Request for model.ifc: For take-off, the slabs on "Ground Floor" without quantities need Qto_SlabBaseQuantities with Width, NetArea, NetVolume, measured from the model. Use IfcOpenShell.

First a look at what the model holds.

```python
import ifcopenshell
import ifcopenshell.util.element
import ifcopenshell.util.unit

model = ifcopenshell.open("model.ifc")
print(model.schema)
for unit_type in ("LENGTHUNIT", "AREAUNIT", "VOLUMEUNIT"):
    print(unit_type, ifcopenshell.util.unit.calculate_unit_scale(model, unit_type))
storey = next(s for s in model.by_type("IfcBuildingStorey") if s.Name == "Ground Floor")
slabs = [e for e in ifcopenshell.util.element.get_decomposition(storey) if e.is_a("IfcSlab")]
for e in sorted(slabs, key=lambda e: e.id()):
    print(e.id(), e.is_a(), e.Name, list(ifcopenshell.util.element.get_psets(e, qtos_only=True)), sep=" | ")
```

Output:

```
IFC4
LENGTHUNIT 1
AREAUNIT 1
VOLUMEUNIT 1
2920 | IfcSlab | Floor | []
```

```python
import ifcopenshell
import ifcopenshell.api.pset
import ifcopenshell.geom
import ifcopenshell.util.element
import ifcopenshell.util.shape
import ifcopenshell.util.unit

model = ifcopenshell.open("model.ifc")
unit_scale = ifcopenshell.util.unit.calculate_unit_scale(model)
area_scale = ifcopenshell.util.unit.calculate_unit_scale(model, "AREAUNIT")
volume_scale = ifcopenshell.util.unit.calculate_unit_scale(model, "VOLUMEUNIT")
settings = ifcopenshell.geom.settings()

storey = next(s for s in model.by_type("IfcBuildingStorey") if s.Name == "Ground Floor")
slabs = [e for e in ifcopenshell.util.element.get_decomposition(storey) if e.is_a("IfcSlab")]

for e in sorted(slabs, key=lambda e: e.id()):
    if ifcopenshell.util.element.get_psets(e, qtos_only=True, should_inherit=False):
        continue
    # Geometry comes back in metres, in the element's own axes.
    shape = ifcopenshell.geom.create_shape(settings, e)
    values = {
        "Width": ifcopenshell.util.shape.get_z(shape.geometry) / unit_scale,
        "NetArea": ifcopenshell.util.shape.get_footprint_area(shape.geometry) / area_scale,
        "NetVolume": ifcopenshell.util.shape.get_volume(shape.geometry) / volume_scale,
    }
    qto = ifcopenshell.api.pset.add_qto(model, product=e, name="Qto_SlabBaseQuantities")
    ifcopenshell.api.pset.edit_qto(model, qto=qto, properties=values)
    print(e.id(), {k: round(v, 3) for k, v in values.items()})

model.write("model_updated.ifc")
```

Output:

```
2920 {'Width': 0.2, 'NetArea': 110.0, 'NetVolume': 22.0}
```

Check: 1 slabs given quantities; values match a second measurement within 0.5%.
